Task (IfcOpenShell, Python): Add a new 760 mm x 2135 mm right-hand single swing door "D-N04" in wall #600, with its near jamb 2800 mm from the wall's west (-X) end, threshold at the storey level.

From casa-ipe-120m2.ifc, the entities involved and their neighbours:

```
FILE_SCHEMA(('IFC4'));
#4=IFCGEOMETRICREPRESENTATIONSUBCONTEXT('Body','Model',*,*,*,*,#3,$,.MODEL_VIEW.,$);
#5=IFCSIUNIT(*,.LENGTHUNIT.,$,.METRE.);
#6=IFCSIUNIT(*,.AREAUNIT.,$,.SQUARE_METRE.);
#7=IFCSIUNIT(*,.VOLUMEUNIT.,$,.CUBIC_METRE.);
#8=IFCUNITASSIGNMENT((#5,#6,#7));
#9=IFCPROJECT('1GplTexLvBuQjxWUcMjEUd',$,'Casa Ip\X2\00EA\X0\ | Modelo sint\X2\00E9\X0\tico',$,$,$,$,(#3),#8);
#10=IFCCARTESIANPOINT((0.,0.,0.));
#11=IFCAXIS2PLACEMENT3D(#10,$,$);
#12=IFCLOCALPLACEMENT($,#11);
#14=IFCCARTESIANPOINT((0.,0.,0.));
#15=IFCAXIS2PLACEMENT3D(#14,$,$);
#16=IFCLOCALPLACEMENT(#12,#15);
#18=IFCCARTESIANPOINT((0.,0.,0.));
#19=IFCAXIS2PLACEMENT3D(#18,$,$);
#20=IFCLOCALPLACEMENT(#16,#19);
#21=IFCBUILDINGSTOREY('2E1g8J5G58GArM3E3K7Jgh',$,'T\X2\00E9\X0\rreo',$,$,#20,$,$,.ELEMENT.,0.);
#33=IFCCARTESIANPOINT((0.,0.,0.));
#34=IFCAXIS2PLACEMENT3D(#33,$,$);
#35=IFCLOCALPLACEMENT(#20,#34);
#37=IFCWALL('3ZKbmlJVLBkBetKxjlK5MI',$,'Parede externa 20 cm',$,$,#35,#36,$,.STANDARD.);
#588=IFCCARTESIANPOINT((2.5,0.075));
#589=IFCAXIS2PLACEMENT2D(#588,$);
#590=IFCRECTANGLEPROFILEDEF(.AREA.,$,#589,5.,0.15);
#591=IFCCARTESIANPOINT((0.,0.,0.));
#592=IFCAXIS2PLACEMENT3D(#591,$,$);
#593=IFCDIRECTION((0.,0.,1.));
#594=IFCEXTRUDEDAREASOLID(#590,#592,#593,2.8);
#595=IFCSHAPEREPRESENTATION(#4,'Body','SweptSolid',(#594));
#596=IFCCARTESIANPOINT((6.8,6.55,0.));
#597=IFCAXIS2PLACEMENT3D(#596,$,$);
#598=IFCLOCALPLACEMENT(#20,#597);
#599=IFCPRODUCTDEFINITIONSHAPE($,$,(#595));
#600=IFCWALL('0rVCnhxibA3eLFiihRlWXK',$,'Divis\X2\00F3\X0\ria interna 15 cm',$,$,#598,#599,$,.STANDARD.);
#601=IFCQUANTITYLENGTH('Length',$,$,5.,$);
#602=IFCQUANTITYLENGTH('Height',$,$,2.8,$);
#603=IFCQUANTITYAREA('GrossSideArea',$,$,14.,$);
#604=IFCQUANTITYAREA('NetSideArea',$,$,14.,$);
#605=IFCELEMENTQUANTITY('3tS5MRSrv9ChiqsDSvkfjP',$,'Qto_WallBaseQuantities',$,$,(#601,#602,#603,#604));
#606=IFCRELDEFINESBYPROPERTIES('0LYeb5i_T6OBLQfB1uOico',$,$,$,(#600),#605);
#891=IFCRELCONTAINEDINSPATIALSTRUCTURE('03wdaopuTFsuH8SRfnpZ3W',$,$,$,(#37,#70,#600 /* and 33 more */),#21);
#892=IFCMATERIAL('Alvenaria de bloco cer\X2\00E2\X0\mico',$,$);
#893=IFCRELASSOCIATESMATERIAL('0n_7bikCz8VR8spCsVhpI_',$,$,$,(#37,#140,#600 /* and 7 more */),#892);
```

```python
import numpy as np
import ifcopenshell
import ifcopenshell.api.feature
import ifcopenshell.api.geometry
import ifcopenshell.api.pset
import ifcopenshell.api.root
import ifcopenshell.api.spatial
import ifcopenshell.geom
import ifcopenshell.util.element
import ifcopenshell.util.placement
import ifcopenshell.util.representation
import ifcopenshell.util.shape
import ifcopenshell.util.unit

model = ifcopenshell.open("casa-ipe-120m2.ifc")
unit_scale = ifcopenshell.util.unit.calculate_unit_scale(model)
area_scale = ifcopenshell.util.unit.calculate_unit_scale(model, "AREAUNIT")
settings = ifcopenshell.geom.settings()


def volume(element):
    """Net volume in cubic metres, openings subtracted."""
    shape = ifcopenshell.geom.create_shape(settings, element)
    return ifcopenshell.util.shape.get_volume(shape.geometry)


wall = model.by_guid("0rVCnhxibA3eLFiihRlWXK")
storey = ifcopenshell.util.element.get_container(wall, ifc_class="IfcBuildingStorey")
context = ifcopenshell.util.representation.get_context(model, "Model", "Body", "MODEL_VIEW")
before = volume(wall)

width, height, from_end, sill = 0.76, 2.135, 2.8, 0.0  # metres

# The wall runs along its own X axis, and the end named is its -X end.
wall_shape = ifcopenshell.geom.create_shape(settings, wall)
x, y, z = ifcopenshell.util.shape.get_vertices(wall_shape.geometry).T
start = x.min() + from_end
face, thickness = float(y.min()), float(y.max() - y.min())
wall_matrix = ifcopenshell.util.placement.get_local_placement(wall.ObjectPlacement)
level = ifcopenshell.util.placement.get_local_placement(storey.ObjectPlacement)[2, 3]


def in_wall(x, y):
    """Placement at x, y metres in the wall's axes, at sill height."""
    matrix = wall_matrix.copy()
    matrix[:, 3] = wall_matrix @ np.array([x / unit_scale, y / unit_scale, 0.0, 1.0])
    matrix[2, 3] = level + sill / unit_scale
    return matrix


# Opening: a box that overshoots both wall faces by 50 mm.
opening = ifcopenshell.api.root.create_entity(model, ifc_class="IfcOpeningElement", predefined_type="OPENING")
box = ifcopenshell.api.geometry.add_wall_representation(
    model, context=context, length=width, height=height, thickness=thickness + 0.1
)
ifcopenshell.api.geometry.assign_representation(model, product=opening, representation=box)
ifcopenshell.api.geometry.edit_object_placement(model, product=opening, matrix=in_wall(start, face - 0.05), is_si=False)
ifcopenshell.api.feature.add_feature(model, feature=opening, element=wall)

door = ifcopenshell.api.root.create_entity(model, ifc_class="IfcDoor", name="D-N04", predefined_type="DOOR")
door.OverallWidth, door.OverallHeight = width / unit_scale, height / unit_scale
door.OperationType = "SINGLE_SWING_RIGHT"
body = ifcopenshell.api.geometry.add_door_representation(
    model,
    context=context,
    overall_width=door.OverallWidth,
    overall_height=door.OverallHeight,
    operation_type="SINGLE_SWING_RIGHT",
    lining_properties={"LiningDepth": thickness / unit_scale, "ThresholdDepth": thickness / unit_scale},
)
ifcopenshell.api.geometry.assign_representation(model, product=door, representation=body)
ifcopenshell.api.spatial.assign_container(model, products=[door], relating_structure=storey)
ifcopenshell.api.feature.add_filling(model, opening=opening, element=door)

# The lining spans the wall, so the door starts at the wall face.
ifcopenshell.api.geometry.edit_object_placement(model, product=door, matrix=in_wall(start, face), is_si=False)

after = volume(wall)

# Update the wall's stored quantities.
qto = model.by_id(ifcopenshell.util.element.get_pset(wall, "Qto_WallBaseQuantities", should_inherit=False)["id"])
ifcopenshell.api.pset.edit_qto(model, qto=qto, properties={"NetSideArea": after / thickness / area_scale})

print(f"wall volume {before:.3f} -> {after:.3f} m3")

model.write("casa-ipe-120m2_v2.ifc")
```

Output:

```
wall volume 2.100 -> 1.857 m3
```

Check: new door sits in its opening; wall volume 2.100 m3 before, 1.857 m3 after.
